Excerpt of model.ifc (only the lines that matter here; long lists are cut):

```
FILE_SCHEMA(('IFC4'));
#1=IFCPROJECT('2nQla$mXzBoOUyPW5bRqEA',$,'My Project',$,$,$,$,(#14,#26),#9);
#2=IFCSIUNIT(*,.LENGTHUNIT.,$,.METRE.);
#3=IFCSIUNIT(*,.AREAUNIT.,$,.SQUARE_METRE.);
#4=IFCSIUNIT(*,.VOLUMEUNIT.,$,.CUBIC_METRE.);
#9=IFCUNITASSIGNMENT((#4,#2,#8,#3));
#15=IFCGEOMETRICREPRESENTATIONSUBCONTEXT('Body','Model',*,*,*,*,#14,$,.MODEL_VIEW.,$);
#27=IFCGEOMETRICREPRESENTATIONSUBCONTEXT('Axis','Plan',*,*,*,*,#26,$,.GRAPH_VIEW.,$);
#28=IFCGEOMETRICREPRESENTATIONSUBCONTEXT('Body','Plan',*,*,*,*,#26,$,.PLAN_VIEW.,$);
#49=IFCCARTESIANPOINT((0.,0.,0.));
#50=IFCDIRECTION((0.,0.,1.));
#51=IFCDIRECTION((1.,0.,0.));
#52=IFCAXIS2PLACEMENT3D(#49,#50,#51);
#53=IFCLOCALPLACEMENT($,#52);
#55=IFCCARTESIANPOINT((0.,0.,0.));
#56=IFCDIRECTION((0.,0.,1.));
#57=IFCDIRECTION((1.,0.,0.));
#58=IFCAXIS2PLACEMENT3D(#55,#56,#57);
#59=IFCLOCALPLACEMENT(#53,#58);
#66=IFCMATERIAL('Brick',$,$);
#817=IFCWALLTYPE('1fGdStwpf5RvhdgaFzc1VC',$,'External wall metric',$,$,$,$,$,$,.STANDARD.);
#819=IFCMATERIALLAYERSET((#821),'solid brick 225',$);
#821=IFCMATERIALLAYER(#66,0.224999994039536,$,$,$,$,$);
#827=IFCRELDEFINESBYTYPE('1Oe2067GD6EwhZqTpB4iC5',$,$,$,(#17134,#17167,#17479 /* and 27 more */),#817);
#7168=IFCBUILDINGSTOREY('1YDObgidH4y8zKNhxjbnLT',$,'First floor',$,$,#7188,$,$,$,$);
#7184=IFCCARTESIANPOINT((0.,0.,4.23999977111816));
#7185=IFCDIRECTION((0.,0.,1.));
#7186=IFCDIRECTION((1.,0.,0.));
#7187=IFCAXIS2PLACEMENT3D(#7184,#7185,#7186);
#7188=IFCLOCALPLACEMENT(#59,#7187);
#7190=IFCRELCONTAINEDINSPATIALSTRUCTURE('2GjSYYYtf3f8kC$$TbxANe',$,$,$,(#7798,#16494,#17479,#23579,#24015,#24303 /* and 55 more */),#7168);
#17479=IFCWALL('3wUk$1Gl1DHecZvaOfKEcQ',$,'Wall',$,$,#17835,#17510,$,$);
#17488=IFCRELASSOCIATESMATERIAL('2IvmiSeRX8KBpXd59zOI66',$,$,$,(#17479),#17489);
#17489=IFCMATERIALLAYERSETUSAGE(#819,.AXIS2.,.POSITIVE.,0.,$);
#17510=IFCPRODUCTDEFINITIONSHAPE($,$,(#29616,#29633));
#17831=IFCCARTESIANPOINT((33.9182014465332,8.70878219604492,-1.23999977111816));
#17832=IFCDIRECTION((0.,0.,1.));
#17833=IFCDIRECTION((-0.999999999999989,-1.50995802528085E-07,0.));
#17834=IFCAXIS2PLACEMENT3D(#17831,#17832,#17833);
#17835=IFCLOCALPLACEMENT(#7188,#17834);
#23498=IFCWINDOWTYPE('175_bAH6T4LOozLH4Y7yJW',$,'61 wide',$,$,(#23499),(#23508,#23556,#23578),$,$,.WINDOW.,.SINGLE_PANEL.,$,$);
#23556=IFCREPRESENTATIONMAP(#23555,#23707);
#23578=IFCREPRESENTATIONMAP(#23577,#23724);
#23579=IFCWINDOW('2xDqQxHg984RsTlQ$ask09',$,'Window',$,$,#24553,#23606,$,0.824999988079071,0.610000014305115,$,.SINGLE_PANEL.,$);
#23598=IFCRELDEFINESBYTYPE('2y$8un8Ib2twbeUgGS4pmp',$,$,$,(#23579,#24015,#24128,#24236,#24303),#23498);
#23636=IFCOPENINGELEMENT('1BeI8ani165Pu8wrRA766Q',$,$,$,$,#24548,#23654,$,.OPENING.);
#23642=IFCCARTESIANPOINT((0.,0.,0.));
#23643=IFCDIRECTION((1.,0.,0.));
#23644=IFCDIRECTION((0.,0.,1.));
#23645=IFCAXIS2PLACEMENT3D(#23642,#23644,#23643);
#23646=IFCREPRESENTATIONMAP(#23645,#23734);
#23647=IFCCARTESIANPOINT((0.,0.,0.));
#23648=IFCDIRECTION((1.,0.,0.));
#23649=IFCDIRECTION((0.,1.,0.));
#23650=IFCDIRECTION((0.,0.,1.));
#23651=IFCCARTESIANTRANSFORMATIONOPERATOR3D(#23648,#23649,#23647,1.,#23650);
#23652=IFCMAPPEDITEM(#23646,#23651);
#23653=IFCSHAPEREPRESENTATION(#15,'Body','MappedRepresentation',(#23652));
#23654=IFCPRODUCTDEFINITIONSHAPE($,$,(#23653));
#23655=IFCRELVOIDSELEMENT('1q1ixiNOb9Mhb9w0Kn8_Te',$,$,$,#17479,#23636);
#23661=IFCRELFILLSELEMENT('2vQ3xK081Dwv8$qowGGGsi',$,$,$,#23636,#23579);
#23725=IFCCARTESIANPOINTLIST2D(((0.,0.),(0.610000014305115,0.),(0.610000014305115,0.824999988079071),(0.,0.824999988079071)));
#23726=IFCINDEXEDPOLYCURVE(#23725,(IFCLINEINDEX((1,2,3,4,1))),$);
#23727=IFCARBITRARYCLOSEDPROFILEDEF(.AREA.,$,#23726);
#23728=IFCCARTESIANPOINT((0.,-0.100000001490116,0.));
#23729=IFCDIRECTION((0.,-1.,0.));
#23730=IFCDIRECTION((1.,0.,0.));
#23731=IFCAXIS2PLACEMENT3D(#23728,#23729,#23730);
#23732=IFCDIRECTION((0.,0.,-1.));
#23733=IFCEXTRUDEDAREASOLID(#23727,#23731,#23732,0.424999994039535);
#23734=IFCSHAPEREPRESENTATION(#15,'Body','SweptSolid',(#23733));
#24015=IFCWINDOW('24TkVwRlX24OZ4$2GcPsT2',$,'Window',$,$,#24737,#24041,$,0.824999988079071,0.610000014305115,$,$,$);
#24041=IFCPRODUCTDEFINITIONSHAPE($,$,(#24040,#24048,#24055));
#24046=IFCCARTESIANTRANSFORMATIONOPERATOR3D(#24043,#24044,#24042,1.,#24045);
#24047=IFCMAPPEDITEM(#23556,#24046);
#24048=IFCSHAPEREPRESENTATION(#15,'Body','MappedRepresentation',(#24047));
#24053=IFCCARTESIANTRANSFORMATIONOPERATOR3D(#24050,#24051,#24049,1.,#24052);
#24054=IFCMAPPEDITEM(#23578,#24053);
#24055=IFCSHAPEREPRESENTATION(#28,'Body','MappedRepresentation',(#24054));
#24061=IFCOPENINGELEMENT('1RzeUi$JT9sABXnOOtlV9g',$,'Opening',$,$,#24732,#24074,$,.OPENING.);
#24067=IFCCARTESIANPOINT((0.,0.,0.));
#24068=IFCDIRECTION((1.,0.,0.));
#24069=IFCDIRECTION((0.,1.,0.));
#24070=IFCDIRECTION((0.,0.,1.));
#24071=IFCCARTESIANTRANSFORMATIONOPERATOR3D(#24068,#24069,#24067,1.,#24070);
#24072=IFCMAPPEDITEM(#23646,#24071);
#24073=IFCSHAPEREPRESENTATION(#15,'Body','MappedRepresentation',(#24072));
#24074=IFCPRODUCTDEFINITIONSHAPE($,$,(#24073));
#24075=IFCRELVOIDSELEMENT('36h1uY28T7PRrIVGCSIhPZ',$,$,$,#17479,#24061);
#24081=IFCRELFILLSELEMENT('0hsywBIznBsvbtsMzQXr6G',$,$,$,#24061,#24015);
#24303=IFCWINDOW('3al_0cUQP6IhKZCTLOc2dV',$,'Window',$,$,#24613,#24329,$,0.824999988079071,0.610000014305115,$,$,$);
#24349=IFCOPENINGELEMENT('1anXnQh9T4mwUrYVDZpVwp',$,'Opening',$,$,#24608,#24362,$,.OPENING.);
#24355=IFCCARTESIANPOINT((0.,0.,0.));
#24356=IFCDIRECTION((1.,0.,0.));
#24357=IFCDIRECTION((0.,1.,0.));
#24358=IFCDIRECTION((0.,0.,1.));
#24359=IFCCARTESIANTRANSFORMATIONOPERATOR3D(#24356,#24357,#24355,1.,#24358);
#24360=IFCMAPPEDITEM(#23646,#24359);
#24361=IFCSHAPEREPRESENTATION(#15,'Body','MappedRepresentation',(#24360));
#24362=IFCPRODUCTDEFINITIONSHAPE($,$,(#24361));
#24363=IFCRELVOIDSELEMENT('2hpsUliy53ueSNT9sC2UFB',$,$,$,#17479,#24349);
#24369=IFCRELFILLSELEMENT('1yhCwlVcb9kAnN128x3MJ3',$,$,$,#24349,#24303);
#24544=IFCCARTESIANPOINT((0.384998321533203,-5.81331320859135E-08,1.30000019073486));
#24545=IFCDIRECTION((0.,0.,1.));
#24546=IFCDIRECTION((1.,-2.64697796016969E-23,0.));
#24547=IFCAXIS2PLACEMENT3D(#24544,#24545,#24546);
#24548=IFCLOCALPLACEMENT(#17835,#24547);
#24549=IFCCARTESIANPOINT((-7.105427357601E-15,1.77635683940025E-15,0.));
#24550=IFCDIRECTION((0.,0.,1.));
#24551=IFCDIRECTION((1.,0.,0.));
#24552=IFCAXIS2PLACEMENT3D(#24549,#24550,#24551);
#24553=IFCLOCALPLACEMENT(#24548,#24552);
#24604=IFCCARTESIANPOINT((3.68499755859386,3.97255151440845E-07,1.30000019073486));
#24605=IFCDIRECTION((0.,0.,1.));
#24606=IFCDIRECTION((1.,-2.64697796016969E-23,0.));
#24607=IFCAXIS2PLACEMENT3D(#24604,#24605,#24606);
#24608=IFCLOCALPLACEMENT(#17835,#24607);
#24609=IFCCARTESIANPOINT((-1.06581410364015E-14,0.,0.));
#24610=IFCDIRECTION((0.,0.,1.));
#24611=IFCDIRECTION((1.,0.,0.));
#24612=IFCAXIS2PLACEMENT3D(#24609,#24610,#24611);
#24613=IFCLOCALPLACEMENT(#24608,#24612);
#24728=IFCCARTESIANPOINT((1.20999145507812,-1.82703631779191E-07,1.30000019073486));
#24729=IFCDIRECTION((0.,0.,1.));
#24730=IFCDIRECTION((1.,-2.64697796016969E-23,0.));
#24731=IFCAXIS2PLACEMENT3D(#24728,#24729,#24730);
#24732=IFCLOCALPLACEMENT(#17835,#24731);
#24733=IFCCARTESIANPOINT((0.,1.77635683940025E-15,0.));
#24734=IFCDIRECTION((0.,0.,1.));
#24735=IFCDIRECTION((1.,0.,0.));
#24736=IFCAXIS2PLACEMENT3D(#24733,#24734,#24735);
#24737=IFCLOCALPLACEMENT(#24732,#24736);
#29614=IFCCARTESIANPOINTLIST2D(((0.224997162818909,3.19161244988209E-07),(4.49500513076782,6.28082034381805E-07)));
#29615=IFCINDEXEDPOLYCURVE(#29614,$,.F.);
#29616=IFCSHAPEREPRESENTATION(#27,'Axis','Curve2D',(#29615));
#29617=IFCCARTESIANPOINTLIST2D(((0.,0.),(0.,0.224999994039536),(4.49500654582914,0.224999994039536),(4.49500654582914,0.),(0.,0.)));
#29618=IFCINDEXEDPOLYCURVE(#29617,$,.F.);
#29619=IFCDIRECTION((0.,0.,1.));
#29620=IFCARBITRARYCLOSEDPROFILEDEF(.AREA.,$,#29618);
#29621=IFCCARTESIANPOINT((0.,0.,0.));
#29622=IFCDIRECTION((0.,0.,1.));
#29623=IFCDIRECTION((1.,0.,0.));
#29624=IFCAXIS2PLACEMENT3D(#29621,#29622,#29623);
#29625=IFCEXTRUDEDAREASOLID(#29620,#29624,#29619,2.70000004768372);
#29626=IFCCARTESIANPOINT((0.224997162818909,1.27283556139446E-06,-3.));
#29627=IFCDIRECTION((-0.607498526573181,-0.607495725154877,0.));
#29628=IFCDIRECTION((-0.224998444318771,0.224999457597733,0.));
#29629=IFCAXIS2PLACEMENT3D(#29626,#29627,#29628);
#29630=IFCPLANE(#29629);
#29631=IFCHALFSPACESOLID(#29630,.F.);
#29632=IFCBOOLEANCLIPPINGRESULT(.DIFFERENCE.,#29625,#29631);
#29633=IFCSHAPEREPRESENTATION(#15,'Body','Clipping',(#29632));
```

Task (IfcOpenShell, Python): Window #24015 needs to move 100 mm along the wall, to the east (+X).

```python
import ifcopenshell
import ifcopenshell.api.geometry
import ifcopenshell.util.placement
import ifcopenshell.util.unit

model = ifcopenshell.open("model.ifc")
unit_scale = ifcopenshell.util.unit.calculate_unit_scale(model)

window = model.by_guid("24TkVwRlX24OZ4$2GcPsT2")
opening = window.FillsVoids[0].RelatingOpeningElement
wall = opening.VoidsElements[0].RelatingBuildingElement

wall_matrix = ifcopenshell.util.placement.get_local_placement(wall.ObjectPlacement)
shift = wall_matrix[:3, 0] * -0.1 / unit_scale
before = ifcopenshell.util.placement.get_local_placement(window.ObjectPlacement)[:3, 3].copy()

# The window is placed relative to its opening, so it follows when the opening moves.
matrix = ifcopenshell.util.placement.get_local_placement(opening.ObjectPlacement)
matrix[:3, 3] += shift
ifcopenshell.api.geometry.edit_object_placement(
    model, product=opening, matrix=matrix, is_si=False, should_transform_children=True
)

after = ifcopenshell.util.placement.get_local_placement(window.ObjectPlacement)[:3, 3]
print("window moved by", (after - before).round(3) + 0.0)

model.write("model_edited.ifc")
```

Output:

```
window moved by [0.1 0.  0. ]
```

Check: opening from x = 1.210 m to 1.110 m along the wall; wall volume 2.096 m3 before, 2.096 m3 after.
